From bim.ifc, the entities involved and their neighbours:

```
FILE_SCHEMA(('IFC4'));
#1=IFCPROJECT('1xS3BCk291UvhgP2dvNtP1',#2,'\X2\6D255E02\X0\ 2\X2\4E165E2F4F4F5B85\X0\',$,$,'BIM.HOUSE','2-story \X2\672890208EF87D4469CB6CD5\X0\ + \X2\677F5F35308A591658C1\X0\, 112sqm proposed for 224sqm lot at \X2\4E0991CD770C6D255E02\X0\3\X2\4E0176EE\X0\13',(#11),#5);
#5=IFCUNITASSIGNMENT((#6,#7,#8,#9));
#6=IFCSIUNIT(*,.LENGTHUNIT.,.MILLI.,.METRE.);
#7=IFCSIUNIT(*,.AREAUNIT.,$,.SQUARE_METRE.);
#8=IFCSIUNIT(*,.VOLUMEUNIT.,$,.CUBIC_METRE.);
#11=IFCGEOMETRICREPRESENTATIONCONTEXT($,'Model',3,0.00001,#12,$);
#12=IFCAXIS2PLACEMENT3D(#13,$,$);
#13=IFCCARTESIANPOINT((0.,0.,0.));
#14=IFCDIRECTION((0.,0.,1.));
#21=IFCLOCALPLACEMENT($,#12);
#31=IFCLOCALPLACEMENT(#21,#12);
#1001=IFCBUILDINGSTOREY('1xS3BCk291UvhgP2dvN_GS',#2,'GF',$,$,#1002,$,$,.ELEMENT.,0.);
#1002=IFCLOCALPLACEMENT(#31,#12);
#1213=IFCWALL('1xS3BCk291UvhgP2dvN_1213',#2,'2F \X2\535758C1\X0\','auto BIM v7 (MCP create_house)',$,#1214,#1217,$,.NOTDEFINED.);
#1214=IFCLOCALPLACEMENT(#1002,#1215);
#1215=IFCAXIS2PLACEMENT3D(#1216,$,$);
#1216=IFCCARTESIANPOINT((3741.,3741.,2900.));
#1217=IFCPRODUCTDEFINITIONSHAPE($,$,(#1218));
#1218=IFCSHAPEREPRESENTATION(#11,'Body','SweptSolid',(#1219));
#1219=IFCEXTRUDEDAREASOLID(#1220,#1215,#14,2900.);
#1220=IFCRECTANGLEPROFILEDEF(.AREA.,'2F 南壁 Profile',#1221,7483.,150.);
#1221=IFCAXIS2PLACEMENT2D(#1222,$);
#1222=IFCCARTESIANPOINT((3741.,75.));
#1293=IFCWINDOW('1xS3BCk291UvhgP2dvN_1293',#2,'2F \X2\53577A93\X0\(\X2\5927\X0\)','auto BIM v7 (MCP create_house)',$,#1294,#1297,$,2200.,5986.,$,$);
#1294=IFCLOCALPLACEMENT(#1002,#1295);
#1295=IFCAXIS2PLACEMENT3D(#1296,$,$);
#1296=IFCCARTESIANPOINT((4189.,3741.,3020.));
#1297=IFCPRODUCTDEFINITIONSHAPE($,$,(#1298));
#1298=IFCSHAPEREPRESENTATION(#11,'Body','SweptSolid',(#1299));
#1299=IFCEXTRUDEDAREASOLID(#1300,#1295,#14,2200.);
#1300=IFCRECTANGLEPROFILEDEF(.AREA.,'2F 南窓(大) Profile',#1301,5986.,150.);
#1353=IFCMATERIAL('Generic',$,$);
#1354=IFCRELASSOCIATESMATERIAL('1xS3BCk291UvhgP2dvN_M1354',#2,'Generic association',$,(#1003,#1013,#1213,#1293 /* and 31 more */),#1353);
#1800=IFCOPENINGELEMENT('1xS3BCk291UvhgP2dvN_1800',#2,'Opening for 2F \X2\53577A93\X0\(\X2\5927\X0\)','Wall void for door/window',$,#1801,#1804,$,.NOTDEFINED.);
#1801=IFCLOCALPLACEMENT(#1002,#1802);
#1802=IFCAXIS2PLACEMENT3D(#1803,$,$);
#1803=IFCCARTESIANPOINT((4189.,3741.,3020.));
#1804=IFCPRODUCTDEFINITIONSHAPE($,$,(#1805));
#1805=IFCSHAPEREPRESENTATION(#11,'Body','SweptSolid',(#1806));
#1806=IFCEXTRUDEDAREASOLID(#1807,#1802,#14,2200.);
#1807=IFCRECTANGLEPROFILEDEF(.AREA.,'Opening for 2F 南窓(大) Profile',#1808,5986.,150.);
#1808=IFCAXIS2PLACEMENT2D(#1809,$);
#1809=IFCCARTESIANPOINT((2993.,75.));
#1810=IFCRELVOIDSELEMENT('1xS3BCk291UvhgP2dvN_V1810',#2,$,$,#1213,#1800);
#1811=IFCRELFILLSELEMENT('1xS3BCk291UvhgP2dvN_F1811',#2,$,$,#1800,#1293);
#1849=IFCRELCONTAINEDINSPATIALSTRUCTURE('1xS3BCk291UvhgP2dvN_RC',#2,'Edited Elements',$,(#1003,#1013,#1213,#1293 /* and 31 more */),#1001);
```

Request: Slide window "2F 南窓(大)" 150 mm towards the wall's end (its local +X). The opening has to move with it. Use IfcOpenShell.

```python
import ifcopenshell
import ifcopenshell.api.geometry
import ifcopenshell.util.placement

model = ifcopenshell.open("bim.ifc")

window = model.by_guid("1xS3BCk291UvhgP2dvN_1293")
opening = window.FillsVoids[0].RelatingOpeningElement
wall = opening.VoidsElements[0].RelatingBuildingElement

wall_matrix = ifcopenshell.util.placement.get_local_placement(wall.ObjectPlacement)
shift = wall_matrix[:3, 0] * 150.0
before = ifcopenshell.util.placement.get_local_placement(window.ObjectPlacement)[:3, 3].copy()

# The window is not placed relative to its opening, so move both.
for product in (opening, window):
    matrix = ifcopenshell.util.placement.get_local_placement(product.ObjectPlacement)
    matrix[:3, 3] += shift
    ifcopenshell.api.geometry.edit_object_placement(model, product=product, matrix=matrix, is_si=False)

after = ifcopenshell.util.placement.get_local_placement(window.ObjectPlacement)[:3, 3]
print("window moved by", (after - before).round(3) + 0.0)

model.write("bim_v2.ifc")
```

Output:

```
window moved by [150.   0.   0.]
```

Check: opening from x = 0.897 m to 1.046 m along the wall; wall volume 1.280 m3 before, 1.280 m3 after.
